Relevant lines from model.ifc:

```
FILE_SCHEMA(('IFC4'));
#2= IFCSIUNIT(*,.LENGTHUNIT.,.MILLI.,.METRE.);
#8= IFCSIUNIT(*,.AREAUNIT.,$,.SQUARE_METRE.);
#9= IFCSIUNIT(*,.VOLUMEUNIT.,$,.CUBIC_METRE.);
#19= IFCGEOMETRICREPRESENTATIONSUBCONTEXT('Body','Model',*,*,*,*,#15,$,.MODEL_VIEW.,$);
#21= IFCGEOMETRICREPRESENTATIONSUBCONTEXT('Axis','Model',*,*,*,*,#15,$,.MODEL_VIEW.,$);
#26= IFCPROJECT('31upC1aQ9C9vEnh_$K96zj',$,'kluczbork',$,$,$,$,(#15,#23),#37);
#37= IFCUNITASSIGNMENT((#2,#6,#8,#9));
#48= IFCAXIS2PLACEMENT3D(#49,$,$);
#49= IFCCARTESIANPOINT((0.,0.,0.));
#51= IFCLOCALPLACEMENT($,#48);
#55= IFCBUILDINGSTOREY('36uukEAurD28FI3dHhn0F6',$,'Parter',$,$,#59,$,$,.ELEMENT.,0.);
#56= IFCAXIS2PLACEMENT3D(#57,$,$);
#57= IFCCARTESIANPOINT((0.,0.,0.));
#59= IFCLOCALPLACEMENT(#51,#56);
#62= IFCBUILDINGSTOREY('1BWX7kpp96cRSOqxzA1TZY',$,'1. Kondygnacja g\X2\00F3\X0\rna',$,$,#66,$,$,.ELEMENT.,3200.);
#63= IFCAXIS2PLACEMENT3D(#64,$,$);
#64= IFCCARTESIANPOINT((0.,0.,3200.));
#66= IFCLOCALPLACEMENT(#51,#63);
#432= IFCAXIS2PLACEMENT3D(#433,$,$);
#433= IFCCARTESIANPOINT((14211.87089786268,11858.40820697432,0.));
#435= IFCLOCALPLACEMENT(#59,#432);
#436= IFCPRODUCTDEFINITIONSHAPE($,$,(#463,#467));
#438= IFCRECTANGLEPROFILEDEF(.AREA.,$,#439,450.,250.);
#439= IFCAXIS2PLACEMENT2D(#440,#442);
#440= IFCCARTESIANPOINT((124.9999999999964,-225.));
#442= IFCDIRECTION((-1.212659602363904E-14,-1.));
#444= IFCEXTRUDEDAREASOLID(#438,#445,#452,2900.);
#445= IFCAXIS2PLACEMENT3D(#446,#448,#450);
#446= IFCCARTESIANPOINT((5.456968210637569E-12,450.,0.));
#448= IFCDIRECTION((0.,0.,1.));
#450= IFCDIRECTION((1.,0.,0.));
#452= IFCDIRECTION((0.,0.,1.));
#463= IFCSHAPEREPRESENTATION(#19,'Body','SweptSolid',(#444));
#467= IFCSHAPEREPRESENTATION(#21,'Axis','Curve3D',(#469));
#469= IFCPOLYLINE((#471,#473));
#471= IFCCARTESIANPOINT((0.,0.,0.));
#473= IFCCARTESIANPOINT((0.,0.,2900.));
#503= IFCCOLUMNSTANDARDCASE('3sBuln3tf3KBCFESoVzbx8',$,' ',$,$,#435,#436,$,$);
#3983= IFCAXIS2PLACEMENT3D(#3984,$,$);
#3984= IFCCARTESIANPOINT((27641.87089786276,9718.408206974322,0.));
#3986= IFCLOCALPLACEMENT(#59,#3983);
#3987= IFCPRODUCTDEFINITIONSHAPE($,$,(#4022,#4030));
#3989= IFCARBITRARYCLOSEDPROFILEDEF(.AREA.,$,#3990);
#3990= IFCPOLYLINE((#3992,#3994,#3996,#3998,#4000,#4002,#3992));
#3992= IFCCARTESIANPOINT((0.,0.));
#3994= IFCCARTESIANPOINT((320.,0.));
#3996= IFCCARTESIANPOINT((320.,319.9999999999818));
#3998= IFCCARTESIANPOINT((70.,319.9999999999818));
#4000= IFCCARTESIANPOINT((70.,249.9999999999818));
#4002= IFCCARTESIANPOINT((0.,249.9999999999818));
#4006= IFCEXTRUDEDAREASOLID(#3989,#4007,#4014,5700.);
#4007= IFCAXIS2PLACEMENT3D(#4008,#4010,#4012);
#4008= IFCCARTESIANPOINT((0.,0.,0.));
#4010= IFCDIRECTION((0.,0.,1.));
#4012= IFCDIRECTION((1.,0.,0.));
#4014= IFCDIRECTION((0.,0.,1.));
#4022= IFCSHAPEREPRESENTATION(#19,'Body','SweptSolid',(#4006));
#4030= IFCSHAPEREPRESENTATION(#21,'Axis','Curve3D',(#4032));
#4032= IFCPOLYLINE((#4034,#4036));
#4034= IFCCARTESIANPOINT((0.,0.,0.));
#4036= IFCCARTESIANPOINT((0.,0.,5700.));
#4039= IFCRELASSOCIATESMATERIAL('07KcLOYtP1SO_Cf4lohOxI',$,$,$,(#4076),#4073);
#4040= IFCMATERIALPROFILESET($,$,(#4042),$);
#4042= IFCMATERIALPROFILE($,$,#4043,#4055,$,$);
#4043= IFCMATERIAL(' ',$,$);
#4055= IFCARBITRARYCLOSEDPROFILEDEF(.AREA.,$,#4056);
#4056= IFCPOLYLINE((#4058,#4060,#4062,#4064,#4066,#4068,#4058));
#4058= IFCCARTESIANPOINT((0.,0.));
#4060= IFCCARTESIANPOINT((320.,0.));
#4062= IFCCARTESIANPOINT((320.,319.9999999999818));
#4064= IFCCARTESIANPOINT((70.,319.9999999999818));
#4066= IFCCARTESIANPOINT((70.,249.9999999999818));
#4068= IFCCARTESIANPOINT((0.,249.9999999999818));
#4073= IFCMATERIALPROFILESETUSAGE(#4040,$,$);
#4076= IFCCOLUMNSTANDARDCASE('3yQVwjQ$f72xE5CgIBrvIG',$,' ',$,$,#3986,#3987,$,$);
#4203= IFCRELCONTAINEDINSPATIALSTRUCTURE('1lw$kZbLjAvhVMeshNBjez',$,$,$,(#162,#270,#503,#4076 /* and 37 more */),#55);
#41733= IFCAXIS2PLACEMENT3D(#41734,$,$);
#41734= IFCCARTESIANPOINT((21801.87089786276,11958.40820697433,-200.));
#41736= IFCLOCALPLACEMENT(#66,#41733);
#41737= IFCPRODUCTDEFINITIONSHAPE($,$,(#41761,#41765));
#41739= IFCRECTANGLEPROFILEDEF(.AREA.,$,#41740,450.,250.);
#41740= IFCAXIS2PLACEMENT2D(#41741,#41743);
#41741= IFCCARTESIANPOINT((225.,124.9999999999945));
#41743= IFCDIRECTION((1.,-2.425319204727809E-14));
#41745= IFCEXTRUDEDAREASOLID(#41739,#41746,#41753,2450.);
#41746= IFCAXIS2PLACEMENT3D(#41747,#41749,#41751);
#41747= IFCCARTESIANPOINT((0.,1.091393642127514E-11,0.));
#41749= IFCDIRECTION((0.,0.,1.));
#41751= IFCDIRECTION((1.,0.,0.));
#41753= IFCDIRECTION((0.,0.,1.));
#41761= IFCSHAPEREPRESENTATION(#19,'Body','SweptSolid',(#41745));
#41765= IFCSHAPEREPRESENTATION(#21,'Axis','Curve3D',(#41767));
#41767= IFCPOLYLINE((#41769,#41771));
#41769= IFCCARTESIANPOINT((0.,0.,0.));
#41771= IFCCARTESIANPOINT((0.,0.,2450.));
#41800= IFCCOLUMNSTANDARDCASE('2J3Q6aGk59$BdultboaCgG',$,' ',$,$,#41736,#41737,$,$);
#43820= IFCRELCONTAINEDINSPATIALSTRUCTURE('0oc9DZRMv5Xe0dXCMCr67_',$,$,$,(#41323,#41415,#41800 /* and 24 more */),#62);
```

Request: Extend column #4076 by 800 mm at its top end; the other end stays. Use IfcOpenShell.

```python
import numpy as np
import ifcopenshell
import ifcopenshell.util.representation

model = ifcopenshell.open("model.ifc")

member = model.by_guid("3yQVwjQ$f72xE5CgIBrvIG")
change = 800.0

# The extrusion runs towards the end named, so only its depth changes.
body = ifcopenshell.util.representation.get_representation(member, "Model", "Body")
solid = body.Items[0]
old_length = solid.Depth
solid.Depth += change

# Move the axis end point with it.
axis = next(r for r in member.Representation.Representations if r.RepresentationIdentifier == "Axis").Items[0]
start, end = (np.array(p.Coordinates) for p in axis.Points)
end = end + (end - start) / np.linalg.norm(end - start) * change
point = model.createIfcCartesianPoint(end.tolist())
axis.Points = [axis.Points[0], point]

print(f"length {old_length:g} -> {solid.Depth:g}")

model.write("model_rev.ifc")
```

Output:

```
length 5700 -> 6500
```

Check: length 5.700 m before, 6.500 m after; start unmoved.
